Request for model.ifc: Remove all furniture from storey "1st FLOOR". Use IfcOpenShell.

First a look at what the model holds.

```python
import ifcopenshell
import ifcopenshell.util.element

model = ifcopenshell.open("model.ifc")
print(model.schema)
storey = next(s for s in model.by_type("IfcBuildingStorey") if s.Name == "1st FLOOR")
furniture = [e for e in ifcopenshell.util.element.get_decomposition(storey) if e.is_a("IfcFurnishingElement")]
seen = {}
for e in furniture:
    element_type = ifcopenshell.util.element.get_type(e)
    name = element_type.Name if element_type not in (None, e) else None
    seen[name] = seen.get(name, 0) + 1
for name, count in sorted(seen.items(), key=str):
    print(count, "x", name)
```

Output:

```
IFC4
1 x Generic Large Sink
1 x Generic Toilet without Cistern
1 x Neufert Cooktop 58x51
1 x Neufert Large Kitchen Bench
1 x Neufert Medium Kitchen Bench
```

```python
import ifcopenshell
import ifcopenshell.api.root
import ifcopenshell.util.element

model = ifcopenshell.open("model.ifc")

storey = next(s for s in model.by_type("IfcBuildingStorey") if s.Name == "1st FLOOR")
furniture = [e for e in ifcopenshell.util.element.get_decomposition(storey) if e.is_a("IfcFurnishingElement")]

for e in furniture:
    ifcopenshell.api.root.remove_product(model, product=e)
print(len(furniture), "removed")

model.write("model_edited.ifc")
```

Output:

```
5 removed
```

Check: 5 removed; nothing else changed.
